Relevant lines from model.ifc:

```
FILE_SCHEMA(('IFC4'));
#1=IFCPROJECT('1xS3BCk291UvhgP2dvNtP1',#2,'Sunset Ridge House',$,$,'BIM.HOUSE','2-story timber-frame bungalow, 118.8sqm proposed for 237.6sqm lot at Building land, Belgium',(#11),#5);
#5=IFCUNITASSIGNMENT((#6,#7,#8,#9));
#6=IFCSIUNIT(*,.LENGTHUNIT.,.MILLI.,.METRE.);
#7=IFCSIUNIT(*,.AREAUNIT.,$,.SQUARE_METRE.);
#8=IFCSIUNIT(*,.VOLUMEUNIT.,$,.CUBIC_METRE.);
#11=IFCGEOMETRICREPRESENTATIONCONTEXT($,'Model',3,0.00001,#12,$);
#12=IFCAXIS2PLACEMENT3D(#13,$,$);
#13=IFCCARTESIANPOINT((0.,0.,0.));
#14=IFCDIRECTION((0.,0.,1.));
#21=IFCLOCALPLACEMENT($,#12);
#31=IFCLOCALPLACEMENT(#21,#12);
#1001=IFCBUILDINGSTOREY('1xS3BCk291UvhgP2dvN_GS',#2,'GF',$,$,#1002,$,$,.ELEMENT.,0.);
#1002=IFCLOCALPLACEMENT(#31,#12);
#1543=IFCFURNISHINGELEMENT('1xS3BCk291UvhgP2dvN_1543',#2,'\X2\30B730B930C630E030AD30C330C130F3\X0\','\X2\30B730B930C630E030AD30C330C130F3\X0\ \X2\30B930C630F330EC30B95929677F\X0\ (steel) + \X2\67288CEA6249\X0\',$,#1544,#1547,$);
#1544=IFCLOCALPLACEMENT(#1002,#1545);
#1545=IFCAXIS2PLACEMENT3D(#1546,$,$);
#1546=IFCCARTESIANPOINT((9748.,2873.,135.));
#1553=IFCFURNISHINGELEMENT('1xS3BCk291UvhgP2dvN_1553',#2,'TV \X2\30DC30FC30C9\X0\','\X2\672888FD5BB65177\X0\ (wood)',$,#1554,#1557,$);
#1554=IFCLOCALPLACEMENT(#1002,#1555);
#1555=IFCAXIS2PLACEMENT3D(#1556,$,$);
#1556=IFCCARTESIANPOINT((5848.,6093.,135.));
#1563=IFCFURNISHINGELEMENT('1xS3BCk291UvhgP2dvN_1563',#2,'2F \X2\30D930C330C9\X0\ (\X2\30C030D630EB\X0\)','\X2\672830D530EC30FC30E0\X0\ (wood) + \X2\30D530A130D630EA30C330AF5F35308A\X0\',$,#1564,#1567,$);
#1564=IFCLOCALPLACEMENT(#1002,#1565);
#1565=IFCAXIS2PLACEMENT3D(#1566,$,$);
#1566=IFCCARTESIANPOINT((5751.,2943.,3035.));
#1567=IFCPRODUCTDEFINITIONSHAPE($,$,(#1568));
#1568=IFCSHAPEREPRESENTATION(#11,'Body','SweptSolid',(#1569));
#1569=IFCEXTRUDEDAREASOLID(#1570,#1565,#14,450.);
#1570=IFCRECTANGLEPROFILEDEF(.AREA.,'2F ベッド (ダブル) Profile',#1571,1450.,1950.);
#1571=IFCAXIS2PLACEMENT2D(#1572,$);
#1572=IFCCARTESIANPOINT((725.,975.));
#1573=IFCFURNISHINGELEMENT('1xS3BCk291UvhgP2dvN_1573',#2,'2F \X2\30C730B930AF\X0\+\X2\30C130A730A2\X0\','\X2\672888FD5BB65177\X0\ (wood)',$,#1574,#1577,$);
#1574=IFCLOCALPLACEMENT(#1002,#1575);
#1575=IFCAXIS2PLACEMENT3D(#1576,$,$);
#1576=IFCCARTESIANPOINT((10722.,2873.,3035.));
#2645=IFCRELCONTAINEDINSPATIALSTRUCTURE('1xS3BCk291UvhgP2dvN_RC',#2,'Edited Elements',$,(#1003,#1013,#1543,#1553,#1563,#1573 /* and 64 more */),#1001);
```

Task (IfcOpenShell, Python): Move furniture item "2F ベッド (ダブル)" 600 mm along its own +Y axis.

```python
import ifcopenshell
import ifcopenshell.api.geometry
import ifcopenshell.util.placement
import ifcopenshell.util.unit

model = ifcopenshell.open("model.ifc")
unit_scale = ifcopenshell.util.unit.calculate_unit_scale(model)

item = model.by_guid("1xS3BCk291UvhgP2dvN_1563")
matrix = ifcopenshell.util.placement.get_local_placement(item.ObjectPlacement)
matrix[:3, 3] += matrix[:3, 1] * 0.6 / unit_scale
ifcopenshell.api.geometry.edit_object_placement(model, product=item, matrix=matrix, is_si=False)

print(ifcopenshell.util.placement.get_local_placement(item.ObjectPlacement).round(3) + 0.0)

model.write("model_rev.ifc")
```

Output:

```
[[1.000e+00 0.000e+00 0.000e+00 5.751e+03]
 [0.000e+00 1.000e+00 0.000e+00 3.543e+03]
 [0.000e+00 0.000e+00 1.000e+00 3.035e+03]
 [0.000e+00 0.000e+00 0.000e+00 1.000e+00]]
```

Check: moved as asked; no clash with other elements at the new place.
